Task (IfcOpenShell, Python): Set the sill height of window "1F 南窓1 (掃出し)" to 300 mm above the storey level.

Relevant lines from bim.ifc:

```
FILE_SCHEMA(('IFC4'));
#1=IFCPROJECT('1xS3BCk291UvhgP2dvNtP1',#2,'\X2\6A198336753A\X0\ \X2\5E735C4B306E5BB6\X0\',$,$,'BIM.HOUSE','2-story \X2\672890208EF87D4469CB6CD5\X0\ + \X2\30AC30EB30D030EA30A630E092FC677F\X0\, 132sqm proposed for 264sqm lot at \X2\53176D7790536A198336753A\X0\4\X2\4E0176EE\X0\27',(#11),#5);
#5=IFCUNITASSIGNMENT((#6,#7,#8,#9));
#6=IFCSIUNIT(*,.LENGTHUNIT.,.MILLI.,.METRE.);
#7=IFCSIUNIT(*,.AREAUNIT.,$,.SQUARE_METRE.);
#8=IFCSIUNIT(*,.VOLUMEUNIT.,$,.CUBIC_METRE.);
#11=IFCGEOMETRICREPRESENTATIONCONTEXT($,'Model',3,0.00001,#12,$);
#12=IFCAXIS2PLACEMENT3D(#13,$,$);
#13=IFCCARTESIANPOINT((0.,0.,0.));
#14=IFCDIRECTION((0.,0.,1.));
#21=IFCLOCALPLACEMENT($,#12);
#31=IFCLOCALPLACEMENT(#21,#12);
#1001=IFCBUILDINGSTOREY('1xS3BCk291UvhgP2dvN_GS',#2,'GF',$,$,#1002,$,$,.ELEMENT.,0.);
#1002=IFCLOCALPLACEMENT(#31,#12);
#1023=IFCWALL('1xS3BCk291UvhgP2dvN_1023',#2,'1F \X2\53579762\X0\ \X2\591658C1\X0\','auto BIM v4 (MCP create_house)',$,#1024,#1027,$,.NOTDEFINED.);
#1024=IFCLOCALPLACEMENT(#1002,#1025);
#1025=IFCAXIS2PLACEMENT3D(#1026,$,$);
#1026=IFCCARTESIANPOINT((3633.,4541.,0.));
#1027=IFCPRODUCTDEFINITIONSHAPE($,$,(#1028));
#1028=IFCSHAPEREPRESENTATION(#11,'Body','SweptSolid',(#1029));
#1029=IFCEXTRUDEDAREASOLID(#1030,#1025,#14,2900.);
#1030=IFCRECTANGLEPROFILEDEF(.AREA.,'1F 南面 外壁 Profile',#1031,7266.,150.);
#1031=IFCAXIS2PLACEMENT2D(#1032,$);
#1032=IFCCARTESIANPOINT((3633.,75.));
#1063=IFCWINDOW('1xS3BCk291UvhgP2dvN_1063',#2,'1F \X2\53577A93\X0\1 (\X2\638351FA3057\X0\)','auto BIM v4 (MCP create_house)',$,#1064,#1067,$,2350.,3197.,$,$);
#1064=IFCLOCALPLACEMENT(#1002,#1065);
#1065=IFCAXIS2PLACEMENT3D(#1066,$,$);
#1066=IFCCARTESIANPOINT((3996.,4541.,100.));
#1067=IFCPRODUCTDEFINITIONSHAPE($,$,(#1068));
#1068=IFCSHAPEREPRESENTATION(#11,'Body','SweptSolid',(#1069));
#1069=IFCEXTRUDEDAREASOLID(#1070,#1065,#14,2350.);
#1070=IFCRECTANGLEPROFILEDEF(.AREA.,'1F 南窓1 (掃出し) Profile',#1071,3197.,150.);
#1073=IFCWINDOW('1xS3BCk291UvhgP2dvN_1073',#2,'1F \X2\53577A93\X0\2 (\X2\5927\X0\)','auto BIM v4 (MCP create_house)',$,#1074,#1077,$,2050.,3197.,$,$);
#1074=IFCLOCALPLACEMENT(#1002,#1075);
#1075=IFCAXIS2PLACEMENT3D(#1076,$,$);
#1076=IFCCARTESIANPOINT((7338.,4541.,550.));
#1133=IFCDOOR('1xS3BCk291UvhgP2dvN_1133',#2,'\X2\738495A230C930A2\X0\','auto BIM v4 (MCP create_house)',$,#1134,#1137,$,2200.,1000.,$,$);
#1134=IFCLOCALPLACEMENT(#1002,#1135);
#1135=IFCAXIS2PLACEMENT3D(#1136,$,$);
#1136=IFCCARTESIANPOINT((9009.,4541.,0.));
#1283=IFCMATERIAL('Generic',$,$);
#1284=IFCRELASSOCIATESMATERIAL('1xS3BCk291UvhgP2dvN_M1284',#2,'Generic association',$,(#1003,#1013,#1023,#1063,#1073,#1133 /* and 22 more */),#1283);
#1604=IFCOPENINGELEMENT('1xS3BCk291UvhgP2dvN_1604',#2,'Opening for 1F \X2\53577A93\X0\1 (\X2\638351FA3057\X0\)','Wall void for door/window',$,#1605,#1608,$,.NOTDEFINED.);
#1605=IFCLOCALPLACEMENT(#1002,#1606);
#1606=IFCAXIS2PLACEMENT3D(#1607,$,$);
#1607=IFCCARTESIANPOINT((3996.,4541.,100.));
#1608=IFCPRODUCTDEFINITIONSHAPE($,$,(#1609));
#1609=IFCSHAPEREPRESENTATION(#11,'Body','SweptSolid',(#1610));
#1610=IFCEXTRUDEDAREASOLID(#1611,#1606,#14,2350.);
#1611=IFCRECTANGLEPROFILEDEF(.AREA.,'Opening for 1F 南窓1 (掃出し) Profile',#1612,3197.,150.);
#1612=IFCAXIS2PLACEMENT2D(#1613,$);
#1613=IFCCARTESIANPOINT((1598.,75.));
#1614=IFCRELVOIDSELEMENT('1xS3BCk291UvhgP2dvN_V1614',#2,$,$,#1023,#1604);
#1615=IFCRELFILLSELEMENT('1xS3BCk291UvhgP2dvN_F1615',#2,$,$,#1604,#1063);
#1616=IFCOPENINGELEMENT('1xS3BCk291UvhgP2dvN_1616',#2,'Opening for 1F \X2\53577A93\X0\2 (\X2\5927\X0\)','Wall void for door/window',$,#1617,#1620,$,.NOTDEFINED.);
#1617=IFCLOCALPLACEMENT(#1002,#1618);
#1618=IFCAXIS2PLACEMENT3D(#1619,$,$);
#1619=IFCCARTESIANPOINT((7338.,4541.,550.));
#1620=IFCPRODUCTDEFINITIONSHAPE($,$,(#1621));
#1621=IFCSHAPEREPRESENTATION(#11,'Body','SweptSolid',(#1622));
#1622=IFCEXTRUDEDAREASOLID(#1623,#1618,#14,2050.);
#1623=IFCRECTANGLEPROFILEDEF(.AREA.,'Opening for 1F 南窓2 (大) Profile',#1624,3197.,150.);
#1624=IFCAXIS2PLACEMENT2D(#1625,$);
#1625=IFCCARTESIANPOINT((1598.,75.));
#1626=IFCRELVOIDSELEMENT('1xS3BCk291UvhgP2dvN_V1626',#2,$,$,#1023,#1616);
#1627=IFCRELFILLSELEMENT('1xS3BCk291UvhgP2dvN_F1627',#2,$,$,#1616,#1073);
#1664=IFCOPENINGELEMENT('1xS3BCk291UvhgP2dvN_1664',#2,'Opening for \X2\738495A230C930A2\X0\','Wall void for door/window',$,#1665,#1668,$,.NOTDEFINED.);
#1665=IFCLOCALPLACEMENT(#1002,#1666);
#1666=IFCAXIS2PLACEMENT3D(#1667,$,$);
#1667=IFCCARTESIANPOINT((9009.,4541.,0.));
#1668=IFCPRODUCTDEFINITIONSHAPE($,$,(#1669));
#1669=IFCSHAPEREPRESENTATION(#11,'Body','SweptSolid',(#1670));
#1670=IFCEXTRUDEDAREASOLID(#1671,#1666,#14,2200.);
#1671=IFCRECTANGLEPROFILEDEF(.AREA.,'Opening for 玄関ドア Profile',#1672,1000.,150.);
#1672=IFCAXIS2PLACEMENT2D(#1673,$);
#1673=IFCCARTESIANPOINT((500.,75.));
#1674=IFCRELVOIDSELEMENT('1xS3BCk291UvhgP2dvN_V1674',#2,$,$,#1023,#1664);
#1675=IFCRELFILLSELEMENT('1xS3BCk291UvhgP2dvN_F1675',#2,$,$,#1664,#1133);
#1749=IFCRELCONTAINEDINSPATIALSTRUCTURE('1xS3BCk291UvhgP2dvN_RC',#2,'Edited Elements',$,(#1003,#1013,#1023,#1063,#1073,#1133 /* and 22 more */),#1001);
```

```python
import numpy as np
import ifcopenshell
import ifcopenshell.api.geometry
import ifcopenshell.geom
import ifcopenshell.util.element
import ifcopenshell.util.placement
import ifcopenshell.util.shape
import ifcopenshell.util.unit

model = ifcopenshell.open("bim.ifc")
unit_scale = ifcopenshell.util.unit.calculate_unit_scale(model)

window = model.by_guid("1xS3BCk291UvhgP2dvN_1063")
opening = window.FillsVoids[0].RelatingOpeningElement
storey = ifcopenshell.util.element.get_container(window, ifc_class="IfcBuildingStorey")
level = ifcopenshell.util.placement.get_local_placement(storey.ObjectPlacement)[2, 3]

# The opening's origin need not be at the sill, so measure its lowest point.
shape = ifcopenshell.geom.create_shape(ifcopenshell.geom.settings(), opening)
bottom = ifcopenshell.util.shape.get_shape_bottom_elevation(shape, shape.geometry) / unit_scale
dz = level + 0.3 / unit_scale - bottom

shift = np.array([0.0, 0.0, dz])
# The window is not placed relative to its opening, so move both.
for product in (opening, window):
    matrix = ifcopenshell.util.placement.get_local_placement(product.ObjectPlacement)
    matrix[:3, 3] += shift
    ifcopenshell.api.geometry.edit_object_placement(model, product=product, matrix=matrix, is_si=False)

print(f"moved by {dz * unit_scale:+.3f} m")

model.write("bim_edited.ifc")
```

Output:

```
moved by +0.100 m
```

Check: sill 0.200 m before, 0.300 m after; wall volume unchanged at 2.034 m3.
